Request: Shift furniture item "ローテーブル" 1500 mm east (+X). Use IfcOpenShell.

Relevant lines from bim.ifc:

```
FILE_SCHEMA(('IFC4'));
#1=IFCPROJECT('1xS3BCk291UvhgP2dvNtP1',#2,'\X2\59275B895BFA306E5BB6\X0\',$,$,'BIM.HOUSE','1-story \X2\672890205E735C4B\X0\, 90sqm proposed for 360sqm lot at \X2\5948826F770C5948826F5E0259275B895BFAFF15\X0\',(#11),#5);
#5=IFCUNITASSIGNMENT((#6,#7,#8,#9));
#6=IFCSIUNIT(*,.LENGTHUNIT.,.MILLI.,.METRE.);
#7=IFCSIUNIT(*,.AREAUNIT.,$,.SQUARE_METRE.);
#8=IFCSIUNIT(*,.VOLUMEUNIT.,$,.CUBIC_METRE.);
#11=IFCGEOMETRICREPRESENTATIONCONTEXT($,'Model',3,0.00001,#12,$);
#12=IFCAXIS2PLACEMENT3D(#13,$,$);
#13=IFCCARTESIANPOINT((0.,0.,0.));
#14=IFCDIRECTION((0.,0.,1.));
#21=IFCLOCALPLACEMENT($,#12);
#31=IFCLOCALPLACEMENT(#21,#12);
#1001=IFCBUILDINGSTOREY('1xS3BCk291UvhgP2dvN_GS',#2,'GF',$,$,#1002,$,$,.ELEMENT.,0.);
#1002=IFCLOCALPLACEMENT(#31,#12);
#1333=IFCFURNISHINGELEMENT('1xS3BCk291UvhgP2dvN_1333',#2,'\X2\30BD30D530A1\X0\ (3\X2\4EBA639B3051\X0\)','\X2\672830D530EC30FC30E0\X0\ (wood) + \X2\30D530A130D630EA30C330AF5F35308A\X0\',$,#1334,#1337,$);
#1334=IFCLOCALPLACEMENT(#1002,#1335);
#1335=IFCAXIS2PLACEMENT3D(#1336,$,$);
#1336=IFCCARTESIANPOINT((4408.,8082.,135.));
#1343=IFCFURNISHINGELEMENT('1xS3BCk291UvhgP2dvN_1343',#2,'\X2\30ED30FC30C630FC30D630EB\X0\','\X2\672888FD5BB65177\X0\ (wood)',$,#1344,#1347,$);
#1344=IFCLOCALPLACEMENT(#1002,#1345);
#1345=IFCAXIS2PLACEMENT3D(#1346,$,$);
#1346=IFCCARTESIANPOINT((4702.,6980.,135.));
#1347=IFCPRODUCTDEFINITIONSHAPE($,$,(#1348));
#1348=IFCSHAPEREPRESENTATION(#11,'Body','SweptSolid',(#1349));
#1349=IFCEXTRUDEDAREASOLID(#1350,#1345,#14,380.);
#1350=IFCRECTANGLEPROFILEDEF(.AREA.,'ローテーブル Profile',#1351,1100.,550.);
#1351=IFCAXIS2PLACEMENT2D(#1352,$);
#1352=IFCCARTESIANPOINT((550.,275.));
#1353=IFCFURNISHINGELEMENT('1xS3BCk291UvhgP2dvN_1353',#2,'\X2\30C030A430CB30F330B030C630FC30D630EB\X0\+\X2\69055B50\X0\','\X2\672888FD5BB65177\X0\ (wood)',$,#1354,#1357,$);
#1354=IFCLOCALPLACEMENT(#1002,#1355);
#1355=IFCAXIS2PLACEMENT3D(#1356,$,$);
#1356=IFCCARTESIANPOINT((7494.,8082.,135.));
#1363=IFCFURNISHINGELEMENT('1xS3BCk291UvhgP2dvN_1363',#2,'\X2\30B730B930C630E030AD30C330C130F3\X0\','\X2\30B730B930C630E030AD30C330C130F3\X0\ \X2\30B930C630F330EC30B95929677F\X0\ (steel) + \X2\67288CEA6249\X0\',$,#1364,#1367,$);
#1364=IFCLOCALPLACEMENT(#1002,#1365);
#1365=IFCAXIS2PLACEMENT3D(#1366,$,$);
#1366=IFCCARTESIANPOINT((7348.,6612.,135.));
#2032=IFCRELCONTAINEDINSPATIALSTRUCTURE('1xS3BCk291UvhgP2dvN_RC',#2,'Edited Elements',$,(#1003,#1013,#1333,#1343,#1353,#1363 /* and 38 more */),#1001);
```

```python
import ifcopenshell
import ifcopenshell.api.geometry
import ifcopenshell.util.placement
import ifcopenshell.util.unit

model = ifcopenshell.open("bim.ifc")
unit_scale = ifcopenshell.util.unit.calculate_unit_scale(model)

item = model.by_guid("1xS3BCk291UvhgP2dvN_1343")
matrix = ifcopenshell.util.placement.get_local_placement(item.ObjectPlacement)
matrix[0, 3] += 1.5 / unit_scale
ifcopenshell.api.geometry.edit_object_placement(model, product=item, matrix=matrix, is_si=False)

print(ifcopenshell.util.placement.get_local_placement(item.ObjectPlacement).round(3) + 0.0)

model.write("bim_rev.ifc")
```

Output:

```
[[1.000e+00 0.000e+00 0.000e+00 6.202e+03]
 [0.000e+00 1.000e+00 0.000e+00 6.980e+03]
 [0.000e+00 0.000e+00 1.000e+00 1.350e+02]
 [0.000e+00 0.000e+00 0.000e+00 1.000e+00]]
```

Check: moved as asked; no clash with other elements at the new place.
